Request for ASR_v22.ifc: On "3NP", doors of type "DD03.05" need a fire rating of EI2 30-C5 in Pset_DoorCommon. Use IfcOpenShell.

First a look at what the model holds.

```python
import ifcopenshell
import ifcopenshell.util.element

model = ifcopenshell.open("ASR_v22.ifc")
print(model.schema)
storey = next(s for s in model.by_type("IfcBuildingStorey") if s.Name == "3NP")
doors = [e for e in ifcopenshell.util.element.get_decomposition(storey) if e.is_a("IfcDoor")]
seen = {}
for e in doors:
    element_type = ifcopenshell.util.element.get_type(e)
    key = (element_type.Name if element_type != e and element_type else None, ifcopenshell.util.element.get_pset(e, "Pset_DoorCommon", "FireRating"))
    seen[key] = seen.get(key, 0) + 1
for (name, value), count in sorted(seen.items(), key=str):
    print(count, "x", name, "|", value)
```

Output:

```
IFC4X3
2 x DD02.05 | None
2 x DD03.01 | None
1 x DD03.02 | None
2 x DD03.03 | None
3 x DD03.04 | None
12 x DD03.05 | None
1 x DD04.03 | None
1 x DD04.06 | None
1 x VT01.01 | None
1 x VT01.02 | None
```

```python
import ifcopenshell
import ifcopenshell.api.pset
import ifcopenshell.util.element

model = ifcopenshell.open("ASR_v22.ifc")

storey = next(s for s in model.by_type("IfcBuildingStorey") if s.Name == "3NP")
doors = [e for e in ifcopenshell.util.element.get_decomposition(storey) if e.is_a("IfcDoor")]

count = 0
for e in doors:
    element_type = ifcopenshell.util.element.get_type(e)
    if element_type in (None, e) or element_type.Name != "DD03.05":
        continue
    # add_pset returns the element's existing set when there is one.
    pset = ifcopenshell.api.pset.add_pset(model, product=e, name="Pset_DoorCommon")
    ifcopenshell.api.pset.edit_pset(model, pset=pset, properties={"FireRating": "EI2 30-C5"})
    count += 1

print(count, "doors updated")

model.write("ASR_v22_edited.ifc")
```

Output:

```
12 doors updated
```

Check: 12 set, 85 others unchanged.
